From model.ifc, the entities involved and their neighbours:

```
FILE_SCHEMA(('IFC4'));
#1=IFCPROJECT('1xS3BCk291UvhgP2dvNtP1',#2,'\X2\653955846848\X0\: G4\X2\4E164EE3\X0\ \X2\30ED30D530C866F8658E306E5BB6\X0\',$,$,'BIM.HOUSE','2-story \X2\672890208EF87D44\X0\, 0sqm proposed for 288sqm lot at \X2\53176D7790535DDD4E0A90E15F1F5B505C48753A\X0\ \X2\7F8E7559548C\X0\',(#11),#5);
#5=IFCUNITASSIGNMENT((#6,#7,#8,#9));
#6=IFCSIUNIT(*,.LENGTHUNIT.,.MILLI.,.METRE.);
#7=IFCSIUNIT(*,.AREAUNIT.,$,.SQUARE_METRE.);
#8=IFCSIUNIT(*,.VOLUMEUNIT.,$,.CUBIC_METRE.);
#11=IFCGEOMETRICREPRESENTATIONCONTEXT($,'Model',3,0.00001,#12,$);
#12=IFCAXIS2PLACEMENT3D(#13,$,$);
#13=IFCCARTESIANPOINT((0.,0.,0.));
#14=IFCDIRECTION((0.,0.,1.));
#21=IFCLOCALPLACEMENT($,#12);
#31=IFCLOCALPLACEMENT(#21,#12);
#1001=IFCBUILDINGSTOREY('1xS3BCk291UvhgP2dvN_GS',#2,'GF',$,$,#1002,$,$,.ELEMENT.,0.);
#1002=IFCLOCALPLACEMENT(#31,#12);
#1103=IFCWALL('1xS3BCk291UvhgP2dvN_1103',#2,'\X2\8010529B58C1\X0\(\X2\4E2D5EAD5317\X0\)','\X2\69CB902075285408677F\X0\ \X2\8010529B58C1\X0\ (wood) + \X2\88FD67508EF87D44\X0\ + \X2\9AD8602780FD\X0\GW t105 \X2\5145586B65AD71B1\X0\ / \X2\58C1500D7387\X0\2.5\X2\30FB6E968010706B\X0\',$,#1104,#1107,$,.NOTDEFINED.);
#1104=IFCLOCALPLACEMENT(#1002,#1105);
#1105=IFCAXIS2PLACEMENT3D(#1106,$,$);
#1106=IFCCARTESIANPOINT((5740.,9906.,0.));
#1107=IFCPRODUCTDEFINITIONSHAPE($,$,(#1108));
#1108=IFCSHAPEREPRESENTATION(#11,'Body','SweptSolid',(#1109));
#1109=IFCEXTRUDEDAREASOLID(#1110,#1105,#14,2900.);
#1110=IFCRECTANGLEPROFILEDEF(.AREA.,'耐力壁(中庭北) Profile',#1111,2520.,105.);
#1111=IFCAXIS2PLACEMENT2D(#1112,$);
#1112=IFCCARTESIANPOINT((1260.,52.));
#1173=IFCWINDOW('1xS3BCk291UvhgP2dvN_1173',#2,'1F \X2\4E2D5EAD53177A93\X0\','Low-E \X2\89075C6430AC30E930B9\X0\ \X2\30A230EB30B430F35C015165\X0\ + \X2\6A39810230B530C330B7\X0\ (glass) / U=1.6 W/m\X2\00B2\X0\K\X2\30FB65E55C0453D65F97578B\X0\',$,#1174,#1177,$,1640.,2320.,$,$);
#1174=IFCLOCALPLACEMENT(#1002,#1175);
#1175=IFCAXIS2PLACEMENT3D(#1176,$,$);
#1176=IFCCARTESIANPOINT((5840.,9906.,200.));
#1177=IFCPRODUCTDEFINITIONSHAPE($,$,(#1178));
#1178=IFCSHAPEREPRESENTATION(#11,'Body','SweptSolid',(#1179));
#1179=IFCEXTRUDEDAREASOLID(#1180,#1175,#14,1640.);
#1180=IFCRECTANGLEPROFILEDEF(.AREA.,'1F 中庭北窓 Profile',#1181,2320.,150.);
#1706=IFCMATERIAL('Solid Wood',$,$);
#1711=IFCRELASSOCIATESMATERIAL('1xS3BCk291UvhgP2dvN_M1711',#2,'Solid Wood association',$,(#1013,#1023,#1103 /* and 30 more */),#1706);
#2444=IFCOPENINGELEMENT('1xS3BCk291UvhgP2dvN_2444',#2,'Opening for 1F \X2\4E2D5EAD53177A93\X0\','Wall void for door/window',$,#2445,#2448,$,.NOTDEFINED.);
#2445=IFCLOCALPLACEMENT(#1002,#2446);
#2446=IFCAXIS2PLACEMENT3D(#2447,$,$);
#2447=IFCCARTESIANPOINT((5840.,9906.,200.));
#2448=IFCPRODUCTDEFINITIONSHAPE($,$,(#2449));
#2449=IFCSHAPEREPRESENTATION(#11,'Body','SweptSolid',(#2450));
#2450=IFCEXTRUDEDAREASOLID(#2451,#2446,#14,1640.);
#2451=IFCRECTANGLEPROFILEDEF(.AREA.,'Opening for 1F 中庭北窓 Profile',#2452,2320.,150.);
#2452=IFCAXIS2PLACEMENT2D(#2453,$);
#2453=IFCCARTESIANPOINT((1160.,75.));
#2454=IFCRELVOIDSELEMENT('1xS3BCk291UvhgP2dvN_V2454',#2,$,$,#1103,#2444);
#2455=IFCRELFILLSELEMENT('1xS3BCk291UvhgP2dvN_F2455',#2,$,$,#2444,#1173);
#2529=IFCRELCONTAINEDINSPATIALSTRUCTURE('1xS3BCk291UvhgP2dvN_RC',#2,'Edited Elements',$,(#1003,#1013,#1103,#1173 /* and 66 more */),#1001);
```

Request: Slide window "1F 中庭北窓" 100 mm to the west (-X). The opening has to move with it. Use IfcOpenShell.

```python
import ifcopenshell
import ifcopenshell.api.geometry
import ifcopenshell.util.placement
import ifcopenshell.util.unit

model = ifcopenshell.open("model.ifc")
unit_scale = ifcopenshell.util.unit.calculate_unit_scale(model)

window = model.by_guid("1xS3BCk291UvhgP2dvN_1173")
opening = window.FillsVoids[0].RelatingOpeningElement
wall = opening.VoidsElements[0].RelatingBuildingElement

wall_matrix = ifcopenshell.util.placement.get_local_placement(wall.ObjectPlacement)
shift = wall_matrix[:3, 0] * -0.1 / unit_scale
before = ifcopenshell.util.placement.get_local_placement(window.ObjectPlacement)[:3, 3].copy()

# The window is not placed relative to its opening, so move both.
for product in (opening, window):
    matrix = ifcopenshell.util.placement.get_local_placement(product.ObjectPlacement)
    matrix[:3, 3] += shift
    ifcopenshell.api.geometry.edit_object_placement(model, product=product, matrix=matrix, is_si=False)

after = ifcopenshell.util.placement.get_local_placement(window.ObjectPlacement)[:3, 3]
print("window moved by", (after - before).round(3) + 0.0)

model.write("model_edited.ifc")
```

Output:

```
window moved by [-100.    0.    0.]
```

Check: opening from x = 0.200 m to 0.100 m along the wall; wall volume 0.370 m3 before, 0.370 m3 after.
